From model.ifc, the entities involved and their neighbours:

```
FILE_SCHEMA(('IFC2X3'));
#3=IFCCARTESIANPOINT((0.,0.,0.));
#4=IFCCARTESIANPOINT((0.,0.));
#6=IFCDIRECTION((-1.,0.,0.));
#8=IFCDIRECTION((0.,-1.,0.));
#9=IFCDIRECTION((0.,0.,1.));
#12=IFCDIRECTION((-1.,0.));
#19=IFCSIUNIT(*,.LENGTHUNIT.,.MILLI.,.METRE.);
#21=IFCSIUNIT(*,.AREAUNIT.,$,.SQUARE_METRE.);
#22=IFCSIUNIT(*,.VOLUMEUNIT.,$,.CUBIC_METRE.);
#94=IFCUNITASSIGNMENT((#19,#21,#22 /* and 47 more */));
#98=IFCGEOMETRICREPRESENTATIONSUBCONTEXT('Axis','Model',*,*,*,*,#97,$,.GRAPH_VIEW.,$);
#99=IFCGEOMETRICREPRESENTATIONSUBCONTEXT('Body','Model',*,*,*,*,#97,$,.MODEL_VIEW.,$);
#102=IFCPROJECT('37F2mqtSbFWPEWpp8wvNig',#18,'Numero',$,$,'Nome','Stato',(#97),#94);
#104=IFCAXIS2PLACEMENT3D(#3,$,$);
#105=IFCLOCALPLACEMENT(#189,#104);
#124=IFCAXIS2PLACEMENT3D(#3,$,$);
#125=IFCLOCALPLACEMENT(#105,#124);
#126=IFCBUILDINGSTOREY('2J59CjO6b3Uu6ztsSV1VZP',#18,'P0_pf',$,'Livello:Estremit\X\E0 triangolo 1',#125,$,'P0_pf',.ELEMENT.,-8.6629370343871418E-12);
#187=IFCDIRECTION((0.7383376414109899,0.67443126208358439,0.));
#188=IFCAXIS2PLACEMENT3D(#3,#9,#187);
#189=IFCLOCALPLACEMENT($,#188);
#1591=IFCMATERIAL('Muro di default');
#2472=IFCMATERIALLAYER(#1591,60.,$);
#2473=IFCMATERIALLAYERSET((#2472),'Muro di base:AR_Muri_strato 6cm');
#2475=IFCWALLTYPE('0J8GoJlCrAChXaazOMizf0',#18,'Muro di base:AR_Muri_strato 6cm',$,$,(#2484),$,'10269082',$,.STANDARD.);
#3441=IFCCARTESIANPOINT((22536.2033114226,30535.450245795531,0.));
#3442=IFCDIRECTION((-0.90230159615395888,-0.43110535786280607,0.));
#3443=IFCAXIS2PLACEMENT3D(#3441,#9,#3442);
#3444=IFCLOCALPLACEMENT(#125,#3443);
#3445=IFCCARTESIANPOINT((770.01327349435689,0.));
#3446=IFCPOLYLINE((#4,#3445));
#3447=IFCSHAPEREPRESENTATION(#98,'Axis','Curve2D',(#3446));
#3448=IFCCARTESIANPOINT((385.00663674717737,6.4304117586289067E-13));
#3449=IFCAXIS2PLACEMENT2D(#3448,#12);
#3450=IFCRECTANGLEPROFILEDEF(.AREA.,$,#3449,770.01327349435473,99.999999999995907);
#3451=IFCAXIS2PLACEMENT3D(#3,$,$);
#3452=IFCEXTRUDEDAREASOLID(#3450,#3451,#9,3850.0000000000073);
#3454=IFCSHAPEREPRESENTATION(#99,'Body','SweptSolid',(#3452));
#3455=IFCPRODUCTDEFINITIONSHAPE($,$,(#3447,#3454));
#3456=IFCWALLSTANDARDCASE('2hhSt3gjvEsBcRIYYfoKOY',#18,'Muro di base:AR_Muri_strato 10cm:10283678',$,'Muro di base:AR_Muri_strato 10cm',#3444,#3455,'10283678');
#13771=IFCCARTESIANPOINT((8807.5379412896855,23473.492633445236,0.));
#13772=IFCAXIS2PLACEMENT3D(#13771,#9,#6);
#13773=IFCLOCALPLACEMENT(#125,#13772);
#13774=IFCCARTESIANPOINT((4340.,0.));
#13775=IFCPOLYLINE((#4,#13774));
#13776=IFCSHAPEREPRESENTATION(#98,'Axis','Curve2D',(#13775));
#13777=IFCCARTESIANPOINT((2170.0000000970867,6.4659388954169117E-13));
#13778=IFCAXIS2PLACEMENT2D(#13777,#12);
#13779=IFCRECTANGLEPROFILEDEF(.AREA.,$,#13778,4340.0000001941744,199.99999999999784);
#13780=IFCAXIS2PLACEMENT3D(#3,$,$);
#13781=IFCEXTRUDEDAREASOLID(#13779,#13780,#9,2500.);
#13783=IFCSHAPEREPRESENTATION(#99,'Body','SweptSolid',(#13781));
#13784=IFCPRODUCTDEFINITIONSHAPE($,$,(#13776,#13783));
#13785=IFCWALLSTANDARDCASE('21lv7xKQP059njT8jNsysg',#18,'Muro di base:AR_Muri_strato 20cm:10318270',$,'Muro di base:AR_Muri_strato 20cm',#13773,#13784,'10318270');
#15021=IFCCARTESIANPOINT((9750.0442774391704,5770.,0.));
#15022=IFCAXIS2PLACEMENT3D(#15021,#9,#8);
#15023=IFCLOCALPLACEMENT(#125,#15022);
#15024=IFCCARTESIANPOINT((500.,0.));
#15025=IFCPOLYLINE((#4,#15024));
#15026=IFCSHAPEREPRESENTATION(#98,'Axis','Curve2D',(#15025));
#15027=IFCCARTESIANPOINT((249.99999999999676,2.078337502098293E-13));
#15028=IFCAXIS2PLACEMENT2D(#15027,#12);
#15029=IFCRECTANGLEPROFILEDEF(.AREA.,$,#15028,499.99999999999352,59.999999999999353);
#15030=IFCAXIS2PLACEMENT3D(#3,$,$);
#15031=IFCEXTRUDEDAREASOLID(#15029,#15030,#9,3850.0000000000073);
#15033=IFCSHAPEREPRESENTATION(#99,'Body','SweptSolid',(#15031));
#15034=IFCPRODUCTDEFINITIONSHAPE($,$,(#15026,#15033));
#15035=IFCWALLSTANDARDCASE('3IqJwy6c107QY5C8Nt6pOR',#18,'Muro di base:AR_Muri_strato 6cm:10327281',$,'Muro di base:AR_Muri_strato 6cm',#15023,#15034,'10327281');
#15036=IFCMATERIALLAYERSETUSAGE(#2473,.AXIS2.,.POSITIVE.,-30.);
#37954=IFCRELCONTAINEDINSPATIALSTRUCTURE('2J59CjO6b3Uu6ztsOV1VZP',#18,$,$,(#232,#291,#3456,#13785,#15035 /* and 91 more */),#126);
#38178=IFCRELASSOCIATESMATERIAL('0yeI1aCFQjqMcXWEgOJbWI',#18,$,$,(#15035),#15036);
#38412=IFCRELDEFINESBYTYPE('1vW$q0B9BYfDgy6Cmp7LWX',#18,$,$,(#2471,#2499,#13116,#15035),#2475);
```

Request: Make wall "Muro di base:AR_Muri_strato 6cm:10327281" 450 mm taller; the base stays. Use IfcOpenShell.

```python
import ifcopenshell
import ifcopenshell.geom
import ifcopenshell.util.representation
import ifcopenshell.util.shape
import ifcopenshell.util.unit

model = ifcopenshell.open("model.ifc")
unit_scale = ifcopenshell.util.unit.calculate_unit_scale(model)
settings = ifcopenshell.geom.settings()


def volume(element):
    """Net volume in cubic metres, openings subtracted."""
    shape = ifcopenshell.geom.create_shape(settings, element)
    return ifcopenshell.util.shape.get_volume(shape.geometry)


wall = model.by_guid("3IqJwy6c107QY5C8Nt6pOR")
before = volume(wall)

body = ifcopenshell.util.representation.get_representation(wall, "Model", "Body")
solid = body.Items[0]
old_height = solid.Depth
solid.Depth += 0.45 / unit_scale
after = volume(wall)

print(f"height {old_height:g} -> {solid.Depth:g}, volume {before:.3f} -> {after:.3f} m3")

model.write("model-out.ifc")
```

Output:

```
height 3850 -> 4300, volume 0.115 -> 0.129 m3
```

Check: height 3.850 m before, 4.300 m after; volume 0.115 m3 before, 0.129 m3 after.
